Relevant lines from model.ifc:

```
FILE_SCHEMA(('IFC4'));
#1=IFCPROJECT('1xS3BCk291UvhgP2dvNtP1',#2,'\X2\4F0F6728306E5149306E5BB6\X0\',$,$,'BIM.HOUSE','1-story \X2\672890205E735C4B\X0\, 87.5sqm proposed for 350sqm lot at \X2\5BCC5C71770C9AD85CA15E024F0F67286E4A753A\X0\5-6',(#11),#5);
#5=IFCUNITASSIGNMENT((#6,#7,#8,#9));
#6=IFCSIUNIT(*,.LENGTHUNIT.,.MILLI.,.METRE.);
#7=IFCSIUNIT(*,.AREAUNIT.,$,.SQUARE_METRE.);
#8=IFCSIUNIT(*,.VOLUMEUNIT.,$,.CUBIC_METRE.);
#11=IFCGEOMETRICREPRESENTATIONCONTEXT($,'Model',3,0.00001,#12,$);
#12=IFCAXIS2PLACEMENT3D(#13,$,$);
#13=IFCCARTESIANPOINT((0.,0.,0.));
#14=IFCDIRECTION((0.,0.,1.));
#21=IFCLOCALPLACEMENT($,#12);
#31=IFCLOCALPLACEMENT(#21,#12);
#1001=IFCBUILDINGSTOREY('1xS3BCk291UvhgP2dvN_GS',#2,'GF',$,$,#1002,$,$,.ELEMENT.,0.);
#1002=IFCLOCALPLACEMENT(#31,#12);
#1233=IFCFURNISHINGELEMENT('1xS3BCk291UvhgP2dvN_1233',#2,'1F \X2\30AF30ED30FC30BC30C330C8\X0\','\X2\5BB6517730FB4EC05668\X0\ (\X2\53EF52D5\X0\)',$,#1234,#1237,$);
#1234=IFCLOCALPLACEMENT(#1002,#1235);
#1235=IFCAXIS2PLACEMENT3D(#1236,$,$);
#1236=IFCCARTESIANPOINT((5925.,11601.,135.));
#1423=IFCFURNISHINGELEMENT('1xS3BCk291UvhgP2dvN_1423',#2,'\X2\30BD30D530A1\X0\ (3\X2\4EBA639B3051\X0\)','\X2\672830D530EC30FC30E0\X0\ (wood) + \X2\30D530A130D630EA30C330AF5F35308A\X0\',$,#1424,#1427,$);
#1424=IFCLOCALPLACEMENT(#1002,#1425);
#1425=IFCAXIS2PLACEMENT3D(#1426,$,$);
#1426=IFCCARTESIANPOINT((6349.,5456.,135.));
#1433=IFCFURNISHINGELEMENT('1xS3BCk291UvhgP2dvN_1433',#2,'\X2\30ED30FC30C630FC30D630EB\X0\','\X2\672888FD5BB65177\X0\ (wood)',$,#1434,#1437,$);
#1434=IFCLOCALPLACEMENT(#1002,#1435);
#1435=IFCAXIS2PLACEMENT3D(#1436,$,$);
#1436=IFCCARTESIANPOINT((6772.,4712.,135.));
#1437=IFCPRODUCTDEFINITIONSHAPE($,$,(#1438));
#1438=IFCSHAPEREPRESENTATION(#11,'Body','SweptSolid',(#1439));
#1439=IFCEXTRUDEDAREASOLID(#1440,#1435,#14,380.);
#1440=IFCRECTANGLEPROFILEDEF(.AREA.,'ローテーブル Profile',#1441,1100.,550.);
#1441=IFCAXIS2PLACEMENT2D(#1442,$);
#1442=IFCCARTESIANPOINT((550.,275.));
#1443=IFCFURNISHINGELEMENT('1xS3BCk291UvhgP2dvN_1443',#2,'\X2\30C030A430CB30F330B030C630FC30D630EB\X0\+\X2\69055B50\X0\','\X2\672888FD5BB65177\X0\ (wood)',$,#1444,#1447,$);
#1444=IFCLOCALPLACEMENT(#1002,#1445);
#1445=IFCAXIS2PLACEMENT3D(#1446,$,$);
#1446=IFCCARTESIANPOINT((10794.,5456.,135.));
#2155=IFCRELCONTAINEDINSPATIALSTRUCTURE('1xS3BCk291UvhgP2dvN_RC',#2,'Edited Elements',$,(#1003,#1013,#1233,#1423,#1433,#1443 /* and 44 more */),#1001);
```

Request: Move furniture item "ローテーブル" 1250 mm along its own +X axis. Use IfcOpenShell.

```python
import ifcopenshell
import ifcopenshell.api.geometry
import ifcopenshell.util.placement
import ifcopenshell.util.unit

model = ifcopenshell.open("model.ifc")
unit_scale = ifcopenshell.util.unit.calculate_unit_scale(model)

item = model.by_guid("1xS3BCk291UvhgP2dvN_1433")
matrix = ifcopenshell.util.placement.get_local_placement(item.ObjectPlacement)
matrix[:3, 3] += matrix[:3, 0] * 1.25 / unit_scale
ifcopenshell.api.geometry.edit_object_placement(model, product=item, matrix=matrix, is_si=False)

print(ifcopenshell.util.placement.get_local_placement(item.ObjectPlacement).round(3) + 0.0)

model.write("model_updated.ifc")
```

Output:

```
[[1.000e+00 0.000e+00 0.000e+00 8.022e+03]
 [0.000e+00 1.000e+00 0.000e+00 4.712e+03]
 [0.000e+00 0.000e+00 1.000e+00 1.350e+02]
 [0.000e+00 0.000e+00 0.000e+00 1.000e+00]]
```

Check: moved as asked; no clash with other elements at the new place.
